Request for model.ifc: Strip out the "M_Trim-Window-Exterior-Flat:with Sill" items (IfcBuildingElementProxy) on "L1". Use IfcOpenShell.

First a look at what the model holds.

```python
import ifcopenshell
import ifcopenshell.util.element

model = ifcopenshell.open("model.ifc")
print(model.schema)
storey = next(s for s in model.by_type("IfcBuildingStorey") if s.Name == "L1")
proxies = [e for e in ifcopenshell.util.element.get_decomposition(storey) if e.is_a("IfcBuildingElementProxy")]
seen = {}
for e in proxies:
    element_type = ifcopenshell.util.element.get_type(e)
    name = element_type.Name if element_type not in (None, e) else None
    seen[name] = seen.get(name, 0) + 1
for name, count in sorted(seen.items(), key=str):
    print(count, "x", name)
```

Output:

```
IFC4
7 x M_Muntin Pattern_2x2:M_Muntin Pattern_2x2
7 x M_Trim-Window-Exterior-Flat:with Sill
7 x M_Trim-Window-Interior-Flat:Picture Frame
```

```python
import ifcopenshell
import ifcopenshell.api.root
import ifcopenshell.util.element

model = ifcopenshell.open("model.ifc")

storey = next(s for s in model.by_type("IfcBuildingStorey") if s.Name == "L1")
proxies = [e for e in ifcopenshell.util.element.get_decomposition(storey) if e.is_a("IfcBuildingElementProxy")]
targets = [e for e in proxies if (t := ifcopenshell.util.element.get_type(e)) not in (None, e) and t.Name == "M_Trim-Window-Exterior-Flat:with Sill"]

for e in targets:
    ifcopenshell.api.root.remove_product(model, product=e)
print(len(targets), "removed")

model.write("model_v2.ifc")
```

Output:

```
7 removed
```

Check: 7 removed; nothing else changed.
